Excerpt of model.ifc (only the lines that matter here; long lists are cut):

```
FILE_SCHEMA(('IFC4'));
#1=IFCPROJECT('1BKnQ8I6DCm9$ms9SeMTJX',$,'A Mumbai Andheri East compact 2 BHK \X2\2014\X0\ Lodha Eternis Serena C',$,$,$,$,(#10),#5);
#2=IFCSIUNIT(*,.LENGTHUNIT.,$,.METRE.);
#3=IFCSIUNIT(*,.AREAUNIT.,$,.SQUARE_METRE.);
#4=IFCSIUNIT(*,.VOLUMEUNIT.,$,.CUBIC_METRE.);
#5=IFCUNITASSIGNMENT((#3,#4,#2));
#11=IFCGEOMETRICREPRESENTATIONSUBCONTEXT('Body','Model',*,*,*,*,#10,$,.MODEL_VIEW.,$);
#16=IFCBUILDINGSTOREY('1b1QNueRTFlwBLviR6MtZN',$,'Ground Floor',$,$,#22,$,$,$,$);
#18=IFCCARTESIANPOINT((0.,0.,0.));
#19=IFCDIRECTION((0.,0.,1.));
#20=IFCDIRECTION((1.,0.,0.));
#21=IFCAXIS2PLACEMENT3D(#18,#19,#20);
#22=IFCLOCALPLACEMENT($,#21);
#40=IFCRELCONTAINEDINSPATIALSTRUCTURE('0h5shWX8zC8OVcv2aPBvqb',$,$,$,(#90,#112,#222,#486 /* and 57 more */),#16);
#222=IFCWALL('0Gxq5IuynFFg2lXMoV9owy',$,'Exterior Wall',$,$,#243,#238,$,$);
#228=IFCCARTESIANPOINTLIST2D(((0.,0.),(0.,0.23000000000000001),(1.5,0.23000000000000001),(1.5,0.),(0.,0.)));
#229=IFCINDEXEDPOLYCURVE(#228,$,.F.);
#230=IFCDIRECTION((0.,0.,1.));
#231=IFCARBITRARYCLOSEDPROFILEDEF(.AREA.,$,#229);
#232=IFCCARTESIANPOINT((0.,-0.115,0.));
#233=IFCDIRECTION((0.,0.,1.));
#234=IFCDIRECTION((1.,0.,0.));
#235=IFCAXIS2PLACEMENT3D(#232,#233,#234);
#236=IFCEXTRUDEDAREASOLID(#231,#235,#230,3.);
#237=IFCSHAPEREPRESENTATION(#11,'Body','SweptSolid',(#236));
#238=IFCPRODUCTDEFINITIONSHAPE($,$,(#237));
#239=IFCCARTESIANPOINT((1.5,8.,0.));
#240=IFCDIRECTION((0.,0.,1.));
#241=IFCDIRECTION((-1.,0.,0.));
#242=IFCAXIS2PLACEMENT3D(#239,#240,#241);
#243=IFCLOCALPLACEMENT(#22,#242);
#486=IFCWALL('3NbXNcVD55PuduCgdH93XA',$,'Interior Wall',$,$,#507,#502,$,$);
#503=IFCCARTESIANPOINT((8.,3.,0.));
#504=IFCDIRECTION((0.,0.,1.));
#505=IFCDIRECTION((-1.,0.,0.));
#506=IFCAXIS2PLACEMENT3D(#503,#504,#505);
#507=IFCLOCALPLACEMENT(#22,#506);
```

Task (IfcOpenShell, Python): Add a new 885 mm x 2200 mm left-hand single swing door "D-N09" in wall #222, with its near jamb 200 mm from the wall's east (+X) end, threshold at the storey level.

```python
import numpy as np
import ifcopenshell
import ifcopenshell.api.feature
import ifcopenshell.api.geometry
import ifcopenshell.api.root
import ifcopenshell.api.spatial
import ifcopenshell.geom
import ifcopenshell.util.element
import ifcopenshell.util.placement
import ifcopenshell.util.representation
import ifcopenshell.util.shape
import ifcopenshell.util.unit

model = ifcopenshell.open("model.ifc")
unit_scale = ifcopenshell.util.unit.calculate_unit_scale(model)
settings = ifcopenshell.geom.settings()


def volume(element):
    """Net volume in cubic metres, openings subtracted."""
    shape = ifcopenshell.geom.create_shape(settings, element)
    return ifcopenshell.util.shape.get_volume(shape.geometry)


wall = model.by_guid("0Gxq5IuynFFg2lXMoV9owy")
storey = ifcopenshell.util.element.get_container(wall, ifc_class="IfcBuildingStorey")
context = ifcopenshell.util.representation.get_context(model, "Model", "Body", "MODEL_VIEW")
before = volume(wall)

width, height, from_end, sill = 0.885, 2.2, 0.2, 0.0  # metres

# The wall runs along its own X axis, and the end named is its -X end.
wall_shape = ifcopenshell.geom.create_shape(settings, wall)
x, y, z = ifcopenshell.util.shape.get_vertices(wall_shape.geometry).T
start = x.min() + from_end
face, thickness = float(y.min()), float(y.max() - y.min())
wall_matrix = ifcopenshell.util.placement.get_local_placement(wall.ObjectPlacement)
level = ifcopenshell.util.placement.get_local_placement(storey.ObjectPlacement)[2, 3]


def in_wall(x, y):
    """Placement at x, y metres in the wall's axes, at sill height."""
    matrix = wall_matrix.copy()
    matrix[:, 3] = wall_matrix @ np.array([x / unit_scale, y / unit_scale, 0.0, 1.0])
    matrix[2, 3] = level + sill / unit_scale
    return matrix


# Opening: a box that overshoots both wall faces by 50 mm.
opening = ifcopenshell.api.root.create_entity(model, ifc_class="IfcOpeningElement", predefined_type="OPENING")
box = ifcopenshell.api.geometry.add_wall_representation(
    model, context=context, length=width, height=height, thickness=thickness + 0.1
)
ifcopenshell.api.geometry.assign_representation(model, product=opening, representation=box)
ifcopenshell.api.geometry.edit_object_placement(model, product=opening, matrix=in_wall(start, face - 0.05), is_si=False)
ifcopenshell.api.feature.add_feature(model, feature=opening, element=wall)

door = ifcopenshell.api.root.create_entity(model, ifc_class="IfcDoor", name="D-N09", predefined_type="DOOR")
door.OverallWidth, door.OverallHeight = width / unit_scale, height / unit_scale
door.OperationType = "SINGLE_SWING_LEFT"
body = ifcopenshell.api.geometry.add_door_representation(
    model,
    context=context,
    overall_width=door.OverallWidth,
    overall_height=door.OverallHeight,
    operation_type="SINGLE_SWING_LEFT",
    lining_properties={"LiningDepth": thickness / unit_scale, "ThresholdDepth": thickness / unit_scale},
)
ifcopenshell.api.geometry.assign_representation(model, product=door, representation=body)
ifcopenshell.api.spatial.assign_container(model, products=[door], relating_structure=storey)
ifcopenshell.api.feature.add_filling(model, opening=opening, element=door)

# The lining spans the wall, so the door starts at the wall face.
ifcopenshell.api.geometry.edit_object_placement(model, product=door, matrix=in_wall(start, face), is_si=False)

after = volume(wall)

print(f"wall volume {before:.3f} -> {after:.3f} m3")

model.write("model_edited.ifc")
```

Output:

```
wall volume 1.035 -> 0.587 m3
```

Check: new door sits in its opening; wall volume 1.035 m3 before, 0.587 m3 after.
